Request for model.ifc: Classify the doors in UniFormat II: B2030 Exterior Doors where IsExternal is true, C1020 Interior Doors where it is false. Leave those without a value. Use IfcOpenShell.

First a look at what the model holds.

```python
import ifcopenshell
import ifcopenshell.util.element

model = ifcopenshell.open("model.ifc")
print(model.schema)
print("classifications:", [c.Name for c in model.by_type("IfcClassification")])
values = [ifcopenshell.util.element.get_pset(e, "Pset_DoorCommon", "IsExternal") for e in model.by_type("IfcDoor")]
for value in (True, False, None):
    print("IsExternal", value, values.count(value))
```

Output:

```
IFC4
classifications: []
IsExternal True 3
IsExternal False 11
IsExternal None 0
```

```python
import ifcopenshell
import ifcopenshell.api.classification
import ifcopenshell.util.element

model = ifcopenshell.open("model.ifc")

system = ifcopenshell.api.classification.add_classification(model, classification="UniFormat II")

doors = model.by_type("IfcDoor")
external = {e: ifcopenshell.util.element.get_pset(e, "Pset_DoorCommon", "IsExternal") for e in doors}
for flag, code, name in ((True, "B2030", "Exterior Doors"), (False, "C1020", "Interior Doors")):
    products = [e for e in doors if external[e] is flag]
    ifcopenshell.api.classification.add_reference(
        model, products=products, classification=system, identification=code, name=name
    )
    print(code, len(products))

model.write("model_edited.ifc")
```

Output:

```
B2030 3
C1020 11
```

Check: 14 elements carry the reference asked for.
